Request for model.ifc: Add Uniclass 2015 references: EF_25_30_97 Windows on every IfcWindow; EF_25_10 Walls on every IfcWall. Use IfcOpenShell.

First a look at what the model holds.

```python
import ifcopenshell

model = ifcopenshell.open("model.ifc")
print(model.schema)
print("classifications:", [c.Name for c in model.by_type("IfcClassification")])
for ifc_class in ("IfcDoor", "IfcRoof", "IfcStair", "IfcWall", "IfcWindow"):
    print(ifc_class, len(model.by_type(ifc_class)))
```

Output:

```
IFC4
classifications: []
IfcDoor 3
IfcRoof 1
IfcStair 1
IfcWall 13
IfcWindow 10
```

```python
import ifcopenshell
import ifcopenshell.api.classification

model = ifcopenshell.open("model.ifc")

system = ifcopenshell.api.classification.add_classification(model, classification="Uniclass 2015")

codes = {
    "IfcWindow": ("EF_25_30_97", "Windows"),
    "IfcWall": ("EF_25_10", "Walls"),
}
for ifc_class, (code, name) in codes.items():
    products = model.by_type(ifc_class)
    ifcopenshell.api.classification.add_reference(
        model, products=products, classification=system, identification=code, name=name
    )
    print(code, len(products))

model.write("model_updated.ifc")
```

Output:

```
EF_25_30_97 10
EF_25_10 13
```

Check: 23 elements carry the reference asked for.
